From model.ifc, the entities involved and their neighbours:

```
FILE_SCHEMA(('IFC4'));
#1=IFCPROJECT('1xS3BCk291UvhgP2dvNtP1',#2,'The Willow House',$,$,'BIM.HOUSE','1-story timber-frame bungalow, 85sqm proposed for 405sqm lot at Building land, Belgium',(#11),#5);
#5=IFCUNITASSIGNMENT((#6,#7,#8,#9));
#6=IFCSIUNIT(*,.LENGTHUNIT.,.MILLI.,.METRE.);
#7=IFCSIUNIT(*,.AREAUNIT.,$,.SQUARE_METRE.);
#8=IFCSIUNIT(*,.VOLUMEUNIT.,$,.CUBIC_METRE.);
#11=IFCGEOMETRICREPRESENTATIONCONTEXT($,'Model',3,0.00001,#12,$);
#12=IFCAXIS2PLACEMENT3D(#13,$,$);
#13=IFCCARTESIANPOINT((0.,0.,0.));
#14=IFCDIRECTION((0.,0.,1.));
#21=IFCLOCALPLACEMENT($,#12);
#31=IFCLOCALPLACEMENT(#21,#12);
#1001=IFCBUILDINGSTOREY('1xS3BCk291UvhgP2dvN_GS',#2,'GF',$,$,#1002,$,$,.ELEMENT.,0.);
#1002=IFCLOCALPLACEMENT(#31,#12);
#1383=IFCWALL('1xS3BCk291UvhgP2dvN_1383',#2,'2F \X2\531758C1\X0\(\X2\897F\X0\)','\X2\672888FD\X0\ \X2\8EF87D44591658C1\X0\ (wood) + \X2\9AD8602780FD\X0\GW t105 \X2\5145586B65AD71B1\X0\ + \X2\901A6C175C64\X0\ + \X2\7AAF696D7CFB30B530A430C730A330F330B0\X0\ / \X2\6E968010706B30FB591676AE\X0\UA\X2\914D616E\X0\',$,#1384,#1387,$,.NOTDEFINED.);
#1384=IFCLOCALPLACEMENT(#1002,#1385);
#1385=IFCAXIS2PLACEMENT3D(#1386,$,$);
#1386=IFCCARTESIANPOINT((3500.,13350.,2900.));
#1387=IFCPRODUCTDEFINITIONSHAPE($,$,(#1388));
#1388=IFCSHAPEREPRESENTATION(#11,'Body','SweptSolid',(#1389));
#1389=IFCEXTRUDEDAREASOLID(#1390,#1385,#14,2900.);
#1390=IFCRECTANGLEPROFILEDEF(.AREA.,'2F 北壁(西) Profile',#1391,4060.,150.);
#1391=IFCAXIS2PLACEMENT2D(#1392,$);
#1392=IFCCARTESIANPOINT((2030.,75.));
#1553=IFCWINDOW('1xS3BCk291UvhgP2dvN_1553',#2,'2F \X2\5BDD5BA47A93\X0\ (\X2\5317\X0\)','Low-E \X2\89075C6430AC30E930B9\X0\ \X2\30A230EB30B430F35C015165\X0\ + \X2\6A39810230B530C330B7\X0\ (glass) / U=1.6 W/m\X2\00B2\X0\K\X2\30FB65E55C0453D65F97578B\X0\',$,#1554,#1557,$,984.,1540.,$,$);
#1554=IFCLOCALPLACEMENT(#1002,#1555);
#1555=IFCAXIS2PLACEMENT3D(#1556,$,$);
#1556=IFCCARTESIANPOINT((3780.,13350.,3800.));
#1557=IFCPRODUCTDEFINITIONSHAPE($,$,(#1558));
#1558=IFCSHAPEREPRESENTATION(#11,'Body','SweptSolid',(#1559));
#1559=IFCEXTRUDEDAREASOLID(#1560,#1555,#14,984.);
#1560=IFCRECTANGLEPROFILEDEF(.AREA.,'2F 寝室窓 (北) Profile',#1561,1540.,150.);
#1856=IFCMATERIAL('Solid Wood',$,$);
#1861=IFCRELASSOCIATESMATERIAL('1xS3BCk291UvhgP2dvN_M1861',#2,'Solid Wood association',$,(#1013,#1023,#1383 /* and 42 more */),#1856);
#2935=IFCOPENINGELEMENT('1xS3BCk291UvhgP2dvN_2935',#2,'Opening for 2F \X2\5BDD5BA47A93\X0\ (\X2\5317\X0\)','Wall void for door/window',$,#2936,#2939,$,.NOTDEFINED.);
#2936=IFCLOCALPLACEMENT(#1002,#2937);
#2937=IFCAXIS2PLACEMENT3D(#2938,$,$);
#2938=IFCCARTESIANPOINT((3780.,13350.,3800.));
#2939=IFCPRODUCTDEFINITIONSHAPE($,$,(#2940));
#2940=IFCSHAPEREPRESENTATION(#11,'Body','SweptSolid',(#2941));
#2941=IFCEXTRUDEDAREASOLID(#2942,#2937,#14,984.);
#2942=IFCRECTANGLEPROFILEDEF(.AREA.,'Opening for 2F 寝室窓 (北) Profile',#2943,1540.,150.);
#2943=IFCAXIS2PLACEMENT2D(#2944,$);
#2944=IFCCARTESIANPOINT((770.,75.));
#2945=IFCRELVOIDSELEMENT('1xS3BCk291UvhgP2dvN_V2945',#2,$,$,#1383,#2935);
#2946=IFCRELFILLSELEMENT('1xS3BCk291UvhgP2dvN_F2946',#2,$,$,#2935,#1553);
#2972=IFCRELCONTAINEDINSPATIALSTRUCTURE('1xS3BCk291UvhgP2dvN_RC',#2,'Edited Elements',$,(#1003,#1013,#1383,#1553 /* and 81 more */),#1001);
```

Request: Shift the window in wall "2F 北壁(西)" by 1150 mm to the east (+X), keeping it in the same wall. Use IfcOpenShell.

```python
import ifcopenshell
import ifcopenshell.api.geometry
import ifcopenshell.util.placement
import ifcopenshell.util.unit

model = ifcopenshell.open("model.ifc")
unit_scale = ifcopenshell.util.unit.calculate_unit_scale(model)

window = model.by_guid("1xS3BCk291UvhgP2dvN_1553")
opening = window.FillsVoids[0].RelatingOpeningElement
wall = opening.VoidsElements[0].RelatingBuildingElement

wall_matrix = ifcopenshell.util.placement.get_local_placement(wall.ObjectPlacement)
shift = wall_matrix[:3, 0] * 1.15 / unit_scale
before = ifcopenshell.util.placement.get_local_placement(window.ObjectPlacement)[:3, 3].copy()

# The window is not placed relative to its opening, so move both.
for product in (opening, window):
    matrix = ifcopenshell.util.placement.get_local_placement(product.ObjectPlacement)
    matrix[:3, 3] += shift
    ifcopenshell.api.geometry.edit_object_placement(model, product=product, matrix=matrix, is_si=False)

after = ifcopenshell.util.placement.get_local_placement(window.ObjectPlacement)[:3, 3]
print("window moved by", (after - before).round(3) + 0.0)

model.write("model_v2.ifc")
```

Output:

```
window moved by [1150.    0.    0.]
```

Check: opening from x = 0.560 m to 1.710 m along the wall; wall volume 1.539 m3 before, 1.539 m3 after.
